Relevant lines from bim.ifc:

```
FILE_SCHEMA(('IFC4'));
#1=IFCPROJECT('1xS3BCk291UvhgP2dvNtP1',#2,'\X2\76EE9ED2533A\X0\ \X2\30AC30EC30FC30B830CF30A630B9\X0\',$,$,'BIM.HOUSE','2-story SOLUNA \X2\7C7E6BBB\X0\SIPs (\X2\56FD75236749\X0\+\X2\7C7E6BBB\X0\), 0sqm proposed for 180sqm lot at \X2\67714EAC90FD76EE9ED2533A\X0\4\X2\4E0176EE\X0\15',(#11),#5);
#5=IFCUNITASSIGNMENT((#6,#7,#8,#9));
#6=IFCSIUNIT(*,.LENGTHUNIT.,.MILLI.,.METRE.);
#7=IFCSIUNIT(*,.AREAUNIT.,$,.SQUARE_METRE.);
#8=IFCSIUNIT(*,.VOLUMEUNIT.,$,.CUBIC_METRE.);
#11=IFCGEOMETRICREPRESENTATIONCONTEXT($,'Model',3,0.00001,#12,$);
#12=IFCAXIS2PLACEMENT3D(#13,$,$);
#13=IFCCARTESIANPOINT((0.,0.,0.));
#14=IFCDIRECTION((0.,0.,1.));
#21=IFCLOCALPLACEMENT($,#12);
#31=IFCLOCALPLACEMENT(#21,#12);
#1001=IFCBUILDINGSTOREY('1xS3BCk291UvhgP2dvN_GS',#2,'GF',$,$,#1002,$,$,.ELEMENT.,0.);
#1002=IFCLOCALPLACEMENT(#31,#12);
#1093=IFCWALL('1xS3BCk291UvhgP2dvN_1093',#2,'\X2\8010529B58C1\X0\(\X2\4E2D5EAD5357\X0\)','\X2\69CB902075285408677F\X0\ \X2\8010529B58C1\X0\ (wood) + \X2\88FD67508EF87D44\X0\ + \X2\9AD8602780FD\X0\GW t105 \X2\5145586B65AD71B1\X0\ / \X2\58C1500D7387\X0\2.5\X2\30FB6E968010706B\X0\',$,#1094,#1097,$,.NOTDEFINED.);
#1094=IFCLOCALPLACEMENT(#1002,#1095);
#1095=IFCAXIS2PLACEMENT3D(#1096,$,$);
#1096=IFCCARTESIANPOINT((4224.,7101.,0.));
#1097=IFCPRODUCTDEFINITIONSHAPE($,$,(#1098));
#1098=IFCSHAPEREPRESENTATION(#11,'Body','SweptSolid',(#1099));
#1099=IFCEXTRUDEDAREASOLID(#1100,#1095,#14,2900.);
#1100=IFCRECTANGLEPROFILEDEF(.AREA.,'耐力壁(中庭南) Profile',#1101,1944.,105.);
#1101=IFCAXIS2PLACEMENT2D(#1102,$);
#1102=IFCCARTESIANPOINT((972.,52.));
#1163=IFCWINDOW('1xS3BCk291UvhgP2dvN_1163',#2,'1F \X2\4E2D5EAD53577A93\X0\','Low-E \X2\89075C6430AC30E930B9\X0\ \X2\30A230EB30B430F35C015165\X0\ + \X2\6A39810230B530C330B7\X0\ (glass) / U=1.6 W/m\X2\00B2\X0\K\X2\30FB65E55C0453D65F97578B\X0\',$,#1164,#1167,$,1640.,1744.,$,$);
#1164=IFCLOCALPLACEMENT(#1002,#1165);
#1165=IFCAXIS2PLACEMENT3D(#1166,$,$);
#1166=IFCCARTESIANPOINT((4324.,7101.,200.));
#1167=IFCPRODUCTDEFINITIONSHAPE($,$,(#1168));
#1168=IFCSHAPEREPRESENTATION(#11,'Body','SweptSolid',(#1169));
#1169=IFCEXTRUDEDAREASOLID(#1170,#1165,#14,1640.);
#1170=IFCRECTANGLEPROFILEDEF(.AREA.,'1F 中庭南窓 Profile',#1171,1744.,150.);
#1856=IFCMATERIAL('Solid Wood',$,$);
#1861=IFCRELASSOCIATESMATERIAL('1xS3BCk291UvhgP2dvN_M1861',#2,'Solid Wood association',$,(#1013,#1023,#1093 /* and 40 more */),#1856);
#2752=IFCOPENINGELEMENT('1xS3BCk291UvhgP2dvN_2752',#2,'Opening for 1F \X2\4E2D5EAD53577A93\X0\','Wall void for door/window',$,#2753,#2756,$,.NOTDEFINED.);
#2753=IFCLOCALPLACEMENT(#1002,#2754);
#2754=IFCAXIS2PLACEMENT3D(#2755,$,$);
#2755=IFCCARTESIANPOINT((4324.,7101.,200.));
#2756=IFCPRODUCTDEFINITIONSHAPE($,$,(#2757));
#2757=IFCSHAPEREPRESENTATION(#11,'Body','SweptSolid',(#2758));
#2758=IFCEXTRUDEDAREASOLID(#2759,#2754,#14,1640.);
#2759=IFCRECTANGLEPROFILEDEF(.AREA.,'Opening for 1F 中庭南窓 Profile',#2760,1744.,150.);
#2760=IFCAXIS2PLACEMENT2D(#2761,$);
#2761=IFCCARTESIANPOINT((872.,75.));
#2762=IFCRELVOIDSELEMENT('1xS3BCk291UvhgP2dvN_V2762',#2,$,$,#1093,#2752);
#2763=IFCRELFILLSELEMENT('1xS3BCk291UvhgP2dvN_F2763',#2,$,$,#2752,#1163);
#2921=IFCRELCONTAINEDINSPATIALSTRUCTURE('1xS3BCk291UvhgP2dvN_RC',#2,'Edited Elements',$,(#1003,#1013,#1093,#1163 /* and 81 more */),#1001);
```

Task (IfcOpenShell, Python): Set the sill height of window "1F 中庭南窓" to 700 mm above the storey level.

```python
import numpy as np
import ifcopenshell
import ifcopenshell.api.geometry
import ifcopenshell.geom
import ifcopenshell.util.element
import ifcopenshell.util.placement
import ifcopenshell.util.shape
import ifcopenshell.util.unit

model = ifcopenshell.open("bim.ifc")
unit_scale = ifcopenshell.util.unit.calculate_unit_scale(model)

window = model.by_id(1163)
opening = window.FillsVoids[0].RelatingOpeningElement
storey = ifcopenshell.util.element.get_container(window, ifc_class="IfcBuildingStorey")
level = ifcopenshell.util.placement.get_local_placement(storey.ObjectPlacement)[2, 3]

# The opening's origin need not be at the sill, so measure its lowest point.
shape = ifcopenshell.geom.create_shape(ifcopenshell.geom.settings(), opening)
bottom = ifcopenshell.util.shape.get_shape_bottom_elevation(shape, shape.geometry) / unit_scale
dz = level + 700.0 - bottom

shift = np.array([0.0, 0.0, dz])
# The window is not placed relative to its opening, so move both.
for product in (opening, window):
    matrix = ifcopenshell.util.placement.get_local_placement(product.ObjectPlacement)
    matrix[:3, 3] += shift
    ifcopenshell.api.geometry.edit_object_placement(model, product=product, matrix=matrix, is_si=False)

print(f"moved by {dz * unit_scale:+.3f} m")

model.write("bim_v2.ifc")
```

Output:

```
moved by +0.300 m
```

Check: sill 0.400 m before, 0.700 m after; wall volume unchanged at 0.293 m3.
